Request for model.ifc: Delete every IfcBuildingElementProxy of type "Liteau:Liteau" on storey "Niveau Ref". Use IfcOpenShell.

First a look at what the model holds.

```python
import ifcopenshell
import ifcopenshell.util.element

model = ifcopenshell.open("model.ifc")
print(model.schema)
storey = next(s for s in model.by_type("IfcBuildingStorey") if s.Name == "Niveau Ref")
proxies = [e for e in ifcopenshell.util.element.get_decomposition(storey) if e.is_a("IfcBuildingElementProxy")]
seen = {}
for e in proxies:
    element_type = ifcopenshell.util.element.get_type(e)
    name = element_type.Name if element_type not in (None, e) else None
    seen[name] = seen.get(name, 0) + 1
for name, count in sorted(seen.items(), key=str):
    print(count, "x", name)
```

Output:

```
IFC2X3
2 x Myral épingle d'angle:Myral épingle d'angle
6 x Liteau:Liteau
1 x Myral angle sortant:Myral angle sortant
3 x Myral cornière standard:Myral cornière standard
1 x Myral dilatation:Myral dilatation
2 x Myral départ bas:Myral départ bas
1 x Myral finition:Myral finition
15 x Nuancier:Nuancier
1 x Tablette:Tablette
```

```python
import ifcopenshell
import ifcopenshell.api.root
import ifcopenshell.util.element

model = ifcopenshell.open("model.ifc")

storey = next(s for s in model.by_type("IfcBuildingStorey") if s.Name == "Niveau Ref")
proxies = [e for e in ifcopenshell.util.element.get_decomposition(storey) if e.is_a("IfcBuildingElementProxy")]
targets = [e for e in proxies if (t := ifcopenshell.util.element.get_type(e)) not in (None, e) and t.Name == "Liteau:Liteau"]

for e in targets:
    ifcopenshell.api.root.remove_product(model, product=e)
print(len(targets), "removed")

model.write("model_v2.ifc")
```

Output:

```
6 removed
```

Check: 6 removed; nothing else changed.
